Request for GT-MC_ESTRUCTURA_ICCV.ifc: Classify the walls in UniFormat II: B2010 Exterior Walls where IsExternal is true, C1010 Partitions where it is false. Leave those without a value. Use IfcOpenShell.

First a look at what the model holds.

```python
import ifcopenshell
import ifcopenshell.util.element

model = ifcopenshell.open("GT-MC_ESTRUCTURA_ICCV.ifc")
print(model.schema)
print("classifications:", [c.Name for c in model.by_type("IfcClassification")])
values = [ifcopenshell.util.element.get_pset(e, "Pset_WallCommon", "IsExternal") for e in model.by_type("IfcWall")]
for value in (True, False, None):
    print("IsExternal", value, values.count(value))
```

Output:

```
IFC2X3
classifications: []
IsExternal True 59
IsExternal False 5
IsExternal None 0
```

```python
import ifcopenshell
import ifcopenshell.api.classification
import ifcopenshell.util.element

model = ifcopenshell.open("GT-MC_ESTRUCTURA_ICCV.ifc")

# IFC2X3 requires Source and Edition and has no link from the project to the system.
system = model.create_entity("IfcClassification", Source="ASTM", Edition="E1557", Name="UniFormat II")

walls = model.by_type("IfcWall")
external = {e: ifcopenshell.util.element.get_pset(e, "Pset_WallCommon", "IsExternal") for e in walls}
for flag, code, name in ((True, "B2010", "Exterior Walls"), (False, "C1010", "Partitions")):
    products = [e for e in walls if external[e] is flag]
    ifcopenshell.api.classification.add_reference(
        model, products=products, classification=system, identification=code, name=name
    )
    print(code, len(products))

model.write("GT-MC_ESTRUCTURA_ICCV-out.ifc")
```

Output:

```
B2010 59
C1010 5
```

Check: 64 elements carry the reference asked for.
